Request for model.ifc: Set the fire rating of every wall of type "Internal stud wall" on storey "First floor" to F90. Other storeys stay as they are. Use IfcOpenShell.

First a look at what the model holds.

```python
import ifcopenshell
import ifcopenshell.util.element

model = ifcopenshell.open("model.ifc")
print(model.schema)
storey = next(s for s in model.by_type("IfcBuildingStorey") if s.Name == "First floor")
walls = [e for e in ifcopenshell.util.element.get_decomposition(storey) if e.is_a("IfcWall")]
seen = {}
for e in walls:
    element_type = ifcopenshell.util.element.get_type(e)
    key = (element_type.Name if element_type != e and element_type else None, ifcopenshell.util.element.get_pset(e, "Pset_WallCommon", "FireRating"))
    seen[key] = seen.get(key, 0) + 1
for (name, value), count in sorted(seen.items(), key=str):
    print(count, "x", name, "|", value)
```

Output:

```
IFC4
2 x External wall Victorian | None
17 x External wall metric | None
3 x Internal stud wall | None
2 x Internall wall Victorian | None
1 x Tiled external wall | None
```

```python
import ifcopenshell
import ifcopenshell.api.pset
import ifcopenshell.util.element

model = ifcopenshell.open("model.ifc")

storey = next(s for s in model.by_type("IfcBuildingStorey") if s.Name == "First floor")
walls = [e for e in ifcopenshell.util.element.get_decomposition(storey) if e.is_a("IfcWall")]

count = 0
for e in walls:
    element_type = ifcopenshell.util.element.get_type(e)
    if element_type in (None, e) or element_type.Name != "Internal stud wall":
        continue
    # add_pset returns the element's existing set when there is one.
    pset = ifcopenshell.api.pset.add_pset(model, product=e, name="Pset_WallCommon")
    ifcopenshell.api.pset.edit_pset(model, pset=pset, properties={"FireRating": "F90"})
    count += 1

print(count, "walls updated")

model.write("model_rev.ifc")
```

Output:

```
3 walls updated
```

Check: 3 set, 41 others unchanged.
